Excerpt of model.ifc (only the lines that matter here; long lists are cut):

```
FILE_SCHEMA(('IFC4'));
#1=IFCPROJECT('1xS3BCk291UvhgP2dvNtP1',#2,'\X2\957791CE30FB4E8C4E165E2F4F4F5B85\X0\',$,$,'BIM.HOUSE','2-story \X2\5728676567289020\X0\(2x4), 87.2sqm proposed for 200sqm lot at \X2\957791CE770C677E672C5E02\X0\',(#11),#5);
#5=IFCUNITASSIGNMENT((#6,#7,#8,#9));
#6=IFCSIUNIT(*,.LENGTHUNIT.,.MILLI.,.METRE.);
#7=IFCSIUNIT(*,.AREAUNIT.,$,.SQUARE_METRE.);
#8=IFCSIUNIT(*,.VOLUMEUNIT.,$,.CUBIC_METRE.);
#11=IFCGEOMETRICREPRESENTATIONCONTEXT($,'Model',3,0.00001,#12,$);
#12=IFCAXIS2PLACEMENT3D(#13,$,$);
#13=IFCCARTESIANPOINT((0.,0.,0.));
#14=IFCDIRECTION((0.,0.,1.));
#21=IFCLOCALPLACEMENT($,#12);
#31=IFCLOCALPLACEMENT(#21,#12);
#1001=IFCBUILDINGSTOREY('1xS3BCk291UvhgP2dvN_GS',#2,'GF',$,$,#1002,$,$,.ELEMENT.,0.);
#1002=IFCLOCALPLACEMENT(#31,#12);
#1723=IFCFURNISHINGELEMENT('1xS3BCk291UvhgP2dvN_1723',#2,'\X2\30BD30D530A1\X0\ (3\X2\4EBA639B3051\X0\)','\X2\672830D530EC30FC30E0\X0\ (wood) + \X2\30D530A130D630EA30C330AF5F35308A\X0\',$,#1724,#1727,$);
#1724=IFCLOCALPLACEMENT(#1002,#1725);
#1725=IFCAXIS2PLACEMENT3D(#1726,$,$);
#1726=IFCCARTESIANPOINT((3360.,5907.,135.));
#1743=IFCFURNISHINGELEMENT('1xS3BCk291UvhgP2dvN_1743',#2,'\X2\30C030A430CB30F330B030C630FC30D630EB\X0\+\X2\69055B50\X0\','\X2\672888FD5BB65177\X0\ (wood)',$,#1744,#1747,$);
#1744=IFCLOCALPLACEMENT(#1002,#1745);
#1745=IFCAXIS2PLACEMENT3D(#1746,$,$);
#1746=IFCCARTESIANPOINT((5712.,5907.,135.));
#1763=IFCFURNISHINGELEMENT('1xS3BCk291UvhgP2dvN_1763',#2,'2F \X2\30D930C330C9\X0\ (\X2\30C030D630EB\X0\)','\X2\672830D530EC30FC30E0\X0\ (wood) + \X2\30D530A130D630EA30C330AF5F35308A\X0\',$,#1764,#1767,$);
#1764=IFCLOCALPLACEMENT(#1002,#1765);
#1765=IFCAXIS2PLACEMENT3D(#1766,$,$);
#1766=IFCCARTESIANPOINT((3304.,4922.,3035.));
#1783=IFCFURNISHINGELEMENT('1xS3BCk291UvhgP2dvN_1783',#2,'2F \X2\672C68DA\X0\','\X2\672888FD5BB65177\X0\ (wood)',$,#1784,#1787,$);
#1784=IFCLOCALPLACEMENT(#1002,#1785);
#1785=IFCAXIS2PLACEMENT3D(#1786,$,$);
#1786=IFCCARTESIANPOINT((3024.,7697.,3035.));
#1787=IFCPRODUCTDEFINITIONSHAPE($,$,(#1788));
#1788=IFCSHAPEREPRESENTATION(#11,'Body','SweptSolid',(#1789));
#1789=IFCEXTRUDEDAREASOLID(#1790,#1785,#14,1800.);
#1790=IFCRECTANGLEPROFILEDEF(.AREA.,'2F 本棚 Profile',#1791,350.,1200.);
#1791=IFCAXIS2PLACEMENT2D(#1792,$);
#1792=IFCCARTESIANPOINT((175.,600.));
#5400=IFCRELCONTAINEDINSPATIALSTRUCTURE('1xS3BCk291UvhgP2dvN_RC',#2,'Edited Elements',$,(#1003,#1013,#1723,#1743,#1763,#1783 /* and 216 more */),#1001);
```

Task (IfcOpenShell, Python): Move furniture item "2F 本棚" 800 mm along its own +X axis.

```python
import ifcopenshell
import ifcopenshell.api.geometry
import ifcopenshell.util.placement
import ifcopenshell.util.unit

model = ifcopenshell.open("model.ifc")
unit_scale = ifcopenshell.util.unit.calculate_unit_scale(model)

item = model.by_guid("1xS3BCk291UvhgP2dvN_1783")
matrix = ifcopenshell.util.placement.get_local_placement(item.ObjectPlacement)
matrix[:3, 3] += matrix[:3, 0] * 0.8 / unit_scale
ifcopenshell.api.geometry.edit_object_placement(model, product=item, matrix=matrix, is_si=False)

print(ifcopenshell.util.placement.get_local_placement(item.ObjectPlacement).round(3) + 0.0)

model.write("model_rev.ifc")
```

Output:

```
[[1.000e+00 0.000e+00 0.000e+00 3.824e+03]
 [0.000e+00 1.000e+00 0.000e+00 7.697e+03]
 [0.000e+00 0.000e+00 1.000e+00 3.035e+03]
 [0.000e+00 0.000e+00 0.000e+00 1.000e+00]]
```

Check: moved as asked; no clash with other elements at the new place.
